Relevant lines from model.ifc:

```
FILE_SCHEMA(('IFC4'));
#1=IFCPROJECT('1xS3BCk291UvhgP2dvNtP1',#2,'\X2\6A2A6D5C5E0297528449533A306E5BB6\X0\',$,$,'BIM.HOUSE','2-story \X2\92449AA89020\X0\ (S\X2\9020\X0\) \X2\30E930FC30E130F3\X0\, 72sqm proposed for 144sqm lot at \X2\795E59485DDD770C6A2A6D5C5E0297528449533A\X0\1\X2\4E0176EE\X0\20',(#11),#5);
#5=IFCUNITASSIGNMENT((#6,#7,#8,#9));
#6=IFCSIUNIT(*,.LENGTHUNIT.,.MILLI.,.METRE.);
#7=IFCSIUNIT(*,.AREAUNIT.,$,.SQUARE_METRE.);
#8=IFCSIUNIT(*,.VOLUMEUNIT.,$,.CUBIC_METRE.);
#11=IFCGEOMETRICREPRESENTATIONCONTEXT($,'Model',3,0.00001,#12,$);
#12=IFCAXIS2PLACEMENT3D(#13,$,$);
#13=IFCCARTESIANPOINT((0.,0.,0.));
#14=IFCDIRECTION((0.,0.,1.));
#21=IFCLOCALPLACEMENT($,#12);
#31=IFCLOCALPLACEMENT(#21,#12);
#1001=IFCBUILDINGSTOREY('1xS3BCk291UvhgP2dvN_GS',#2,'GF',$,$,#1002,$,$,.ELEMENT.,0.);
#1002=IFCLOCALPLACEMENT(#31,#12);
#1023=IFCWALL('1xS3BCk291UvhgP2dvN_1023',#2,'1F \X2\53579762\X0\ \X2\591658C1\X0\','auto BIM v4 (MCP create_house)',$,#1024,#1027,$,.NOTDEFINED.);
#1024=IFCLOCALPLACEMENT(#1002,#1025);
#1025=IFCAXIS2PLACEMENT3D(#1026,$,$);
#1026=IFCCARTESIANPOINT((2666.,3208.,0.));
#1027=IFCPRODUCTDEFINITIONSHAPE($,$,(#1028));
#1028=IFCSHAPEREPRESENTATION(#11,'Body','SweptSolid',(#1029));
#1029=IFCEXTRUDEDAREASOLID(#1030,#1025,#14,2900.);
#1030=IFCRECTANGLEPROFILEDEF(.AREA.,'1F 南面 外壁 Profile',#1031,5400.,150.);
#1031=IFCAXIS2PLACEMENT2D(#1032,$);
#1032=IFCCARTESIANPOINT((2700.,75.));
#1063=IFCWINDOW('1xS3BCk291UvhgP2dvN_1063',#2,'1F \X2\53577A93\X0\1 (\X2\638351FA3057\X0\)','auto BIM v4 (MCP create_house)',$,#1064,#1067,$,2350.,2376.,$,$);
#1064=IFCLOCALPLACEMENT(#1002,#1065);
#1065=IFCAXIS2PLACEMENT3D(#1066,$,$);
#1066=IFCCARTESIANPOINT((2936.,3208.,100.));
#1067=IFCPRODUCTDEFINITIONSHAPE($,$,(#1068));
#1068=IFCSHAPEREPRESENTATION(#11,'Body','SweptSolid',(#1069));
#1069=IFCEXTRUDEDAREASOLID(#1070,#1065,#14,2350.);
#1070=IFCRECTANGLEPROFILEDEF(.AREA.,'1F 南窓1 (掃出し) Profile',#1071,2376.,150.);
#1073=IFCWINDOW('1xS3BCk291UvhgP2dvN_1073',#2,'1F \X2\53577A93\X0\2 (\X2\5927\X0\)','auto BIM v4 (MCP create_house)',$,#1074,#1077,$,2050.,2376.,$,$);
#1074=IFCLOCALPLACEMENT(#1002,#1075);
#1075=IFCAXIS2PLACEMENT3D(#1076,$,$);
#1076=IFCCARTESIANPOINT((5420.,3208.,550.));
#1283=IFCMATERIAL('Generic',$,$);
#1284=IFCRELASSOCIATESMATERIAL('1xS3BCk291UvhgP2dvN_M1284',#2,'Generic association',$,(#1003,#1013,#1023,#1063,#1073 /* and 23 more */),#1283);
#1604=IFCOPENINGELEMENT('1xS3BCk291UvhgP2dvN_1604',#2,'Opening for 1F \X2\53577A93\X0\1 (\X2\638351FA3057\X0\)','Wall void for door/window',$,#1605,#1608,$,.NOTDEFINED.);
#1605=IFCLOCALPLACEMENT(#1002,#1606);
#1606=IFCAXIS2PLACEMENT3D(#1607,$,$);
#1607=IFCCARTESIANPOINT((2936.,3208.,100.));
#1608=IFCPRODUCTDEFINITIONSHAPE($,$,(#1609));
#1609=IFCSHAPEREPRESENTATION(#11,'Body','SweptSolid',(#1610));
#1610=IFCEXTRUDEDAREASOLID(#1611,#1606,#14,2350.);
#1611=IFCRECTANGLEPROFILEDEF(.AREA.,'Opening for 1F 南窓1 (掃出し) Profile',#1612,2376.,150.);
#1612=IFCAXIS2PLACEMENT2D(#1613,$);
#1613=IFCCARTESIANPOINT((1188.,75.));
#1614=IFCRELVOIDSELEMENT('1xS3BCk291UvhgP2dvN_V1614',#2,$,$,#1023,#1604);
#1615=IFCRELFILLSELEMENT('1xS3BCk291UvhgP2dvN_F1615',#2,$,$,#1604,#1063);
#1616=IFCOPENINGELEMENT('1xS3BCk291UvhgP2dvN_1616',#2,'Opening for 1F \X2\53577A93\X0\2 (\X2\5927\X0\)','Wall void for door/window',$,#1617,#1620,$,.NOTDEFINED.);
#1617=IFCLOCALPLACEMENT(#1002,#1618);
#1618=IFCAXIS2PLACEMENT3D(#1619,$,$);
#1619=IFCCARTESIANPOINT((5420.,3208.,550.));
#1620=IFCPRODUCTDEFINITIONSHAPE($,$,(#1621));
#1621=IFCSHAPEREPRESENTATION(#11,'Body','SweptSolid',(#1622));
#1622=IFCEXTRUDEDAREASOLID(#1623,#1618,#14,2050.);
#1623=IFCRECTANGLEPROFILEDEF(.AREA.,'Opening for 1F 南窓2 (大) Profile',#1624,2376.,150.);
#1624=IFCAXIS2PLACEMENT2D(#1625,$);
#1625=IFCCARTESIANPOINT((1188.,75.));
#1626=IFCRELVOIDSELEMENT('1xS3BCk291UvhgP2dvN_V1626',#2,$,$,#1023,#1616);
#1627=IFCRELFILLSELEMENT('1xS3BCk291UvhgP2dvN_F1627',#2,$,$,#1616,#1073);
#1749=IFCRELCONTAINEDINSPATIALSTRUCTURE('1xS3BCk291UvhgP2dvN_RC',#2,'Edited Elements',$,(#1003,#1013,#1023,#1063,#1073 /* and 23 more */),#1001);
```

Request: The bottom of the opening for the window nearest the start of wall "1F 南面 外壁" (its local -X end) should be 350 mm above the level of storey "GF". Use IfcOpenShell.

```python
import numpy as np
import ifcopenshell
import ifcopenshell.api.geometry
import ifcopenshell.geom
import ifcopenshell.util.element
import ifcopenshell.util.placement
import ifcopenshell.util.shape
import ifcopenshell.util.unit

model = ifcopenshell.open("model.ifc")
unit_scale = ifcopenshell.util.unit.calculate_unit_scale(model)

window = model.by_id(1063)
opening = window.FillsVoids[0].RelatingOpeningElement
storey = ifcopenshell.util.element.get_container(window, ifc_class="IfcBuildingStorey")
level = ifcopenshell.util.placement.get_local_placement(storey.ObjectPlacement)[2, 3]

# The opening's origin need not be at the sill, so measure its lowest point.
shape = ifcopenshell.geom.create_shape(ifcopenshell.geom.settings(), opening)
bottom = ifcopenshell.util.shape.get_shape_bottom_elevation(shape, shape.geometry) / unit_scale
dz = level + 0.35 / unit_scale - bottom

shift = np.array([0.0, 0.0, dz])
# The window is not placed relative to its opening, so move both.
for product in (opening, window):
    matrix = ifcopenshell.util.placement.get_local_placement(product.ObjectPlacement)
    matrix[:3, 3] += shift
    ifcopenshell.api.geometry.edit_object_placement(model, product=product, matrix=matrix, is_si=False)

print(f"moved by {dz * unit_scale:+.3f} m")

model.write("model_updated.ifc")
```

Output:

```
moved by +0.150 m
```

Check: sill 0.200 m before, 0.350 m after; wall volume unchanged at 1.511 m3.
